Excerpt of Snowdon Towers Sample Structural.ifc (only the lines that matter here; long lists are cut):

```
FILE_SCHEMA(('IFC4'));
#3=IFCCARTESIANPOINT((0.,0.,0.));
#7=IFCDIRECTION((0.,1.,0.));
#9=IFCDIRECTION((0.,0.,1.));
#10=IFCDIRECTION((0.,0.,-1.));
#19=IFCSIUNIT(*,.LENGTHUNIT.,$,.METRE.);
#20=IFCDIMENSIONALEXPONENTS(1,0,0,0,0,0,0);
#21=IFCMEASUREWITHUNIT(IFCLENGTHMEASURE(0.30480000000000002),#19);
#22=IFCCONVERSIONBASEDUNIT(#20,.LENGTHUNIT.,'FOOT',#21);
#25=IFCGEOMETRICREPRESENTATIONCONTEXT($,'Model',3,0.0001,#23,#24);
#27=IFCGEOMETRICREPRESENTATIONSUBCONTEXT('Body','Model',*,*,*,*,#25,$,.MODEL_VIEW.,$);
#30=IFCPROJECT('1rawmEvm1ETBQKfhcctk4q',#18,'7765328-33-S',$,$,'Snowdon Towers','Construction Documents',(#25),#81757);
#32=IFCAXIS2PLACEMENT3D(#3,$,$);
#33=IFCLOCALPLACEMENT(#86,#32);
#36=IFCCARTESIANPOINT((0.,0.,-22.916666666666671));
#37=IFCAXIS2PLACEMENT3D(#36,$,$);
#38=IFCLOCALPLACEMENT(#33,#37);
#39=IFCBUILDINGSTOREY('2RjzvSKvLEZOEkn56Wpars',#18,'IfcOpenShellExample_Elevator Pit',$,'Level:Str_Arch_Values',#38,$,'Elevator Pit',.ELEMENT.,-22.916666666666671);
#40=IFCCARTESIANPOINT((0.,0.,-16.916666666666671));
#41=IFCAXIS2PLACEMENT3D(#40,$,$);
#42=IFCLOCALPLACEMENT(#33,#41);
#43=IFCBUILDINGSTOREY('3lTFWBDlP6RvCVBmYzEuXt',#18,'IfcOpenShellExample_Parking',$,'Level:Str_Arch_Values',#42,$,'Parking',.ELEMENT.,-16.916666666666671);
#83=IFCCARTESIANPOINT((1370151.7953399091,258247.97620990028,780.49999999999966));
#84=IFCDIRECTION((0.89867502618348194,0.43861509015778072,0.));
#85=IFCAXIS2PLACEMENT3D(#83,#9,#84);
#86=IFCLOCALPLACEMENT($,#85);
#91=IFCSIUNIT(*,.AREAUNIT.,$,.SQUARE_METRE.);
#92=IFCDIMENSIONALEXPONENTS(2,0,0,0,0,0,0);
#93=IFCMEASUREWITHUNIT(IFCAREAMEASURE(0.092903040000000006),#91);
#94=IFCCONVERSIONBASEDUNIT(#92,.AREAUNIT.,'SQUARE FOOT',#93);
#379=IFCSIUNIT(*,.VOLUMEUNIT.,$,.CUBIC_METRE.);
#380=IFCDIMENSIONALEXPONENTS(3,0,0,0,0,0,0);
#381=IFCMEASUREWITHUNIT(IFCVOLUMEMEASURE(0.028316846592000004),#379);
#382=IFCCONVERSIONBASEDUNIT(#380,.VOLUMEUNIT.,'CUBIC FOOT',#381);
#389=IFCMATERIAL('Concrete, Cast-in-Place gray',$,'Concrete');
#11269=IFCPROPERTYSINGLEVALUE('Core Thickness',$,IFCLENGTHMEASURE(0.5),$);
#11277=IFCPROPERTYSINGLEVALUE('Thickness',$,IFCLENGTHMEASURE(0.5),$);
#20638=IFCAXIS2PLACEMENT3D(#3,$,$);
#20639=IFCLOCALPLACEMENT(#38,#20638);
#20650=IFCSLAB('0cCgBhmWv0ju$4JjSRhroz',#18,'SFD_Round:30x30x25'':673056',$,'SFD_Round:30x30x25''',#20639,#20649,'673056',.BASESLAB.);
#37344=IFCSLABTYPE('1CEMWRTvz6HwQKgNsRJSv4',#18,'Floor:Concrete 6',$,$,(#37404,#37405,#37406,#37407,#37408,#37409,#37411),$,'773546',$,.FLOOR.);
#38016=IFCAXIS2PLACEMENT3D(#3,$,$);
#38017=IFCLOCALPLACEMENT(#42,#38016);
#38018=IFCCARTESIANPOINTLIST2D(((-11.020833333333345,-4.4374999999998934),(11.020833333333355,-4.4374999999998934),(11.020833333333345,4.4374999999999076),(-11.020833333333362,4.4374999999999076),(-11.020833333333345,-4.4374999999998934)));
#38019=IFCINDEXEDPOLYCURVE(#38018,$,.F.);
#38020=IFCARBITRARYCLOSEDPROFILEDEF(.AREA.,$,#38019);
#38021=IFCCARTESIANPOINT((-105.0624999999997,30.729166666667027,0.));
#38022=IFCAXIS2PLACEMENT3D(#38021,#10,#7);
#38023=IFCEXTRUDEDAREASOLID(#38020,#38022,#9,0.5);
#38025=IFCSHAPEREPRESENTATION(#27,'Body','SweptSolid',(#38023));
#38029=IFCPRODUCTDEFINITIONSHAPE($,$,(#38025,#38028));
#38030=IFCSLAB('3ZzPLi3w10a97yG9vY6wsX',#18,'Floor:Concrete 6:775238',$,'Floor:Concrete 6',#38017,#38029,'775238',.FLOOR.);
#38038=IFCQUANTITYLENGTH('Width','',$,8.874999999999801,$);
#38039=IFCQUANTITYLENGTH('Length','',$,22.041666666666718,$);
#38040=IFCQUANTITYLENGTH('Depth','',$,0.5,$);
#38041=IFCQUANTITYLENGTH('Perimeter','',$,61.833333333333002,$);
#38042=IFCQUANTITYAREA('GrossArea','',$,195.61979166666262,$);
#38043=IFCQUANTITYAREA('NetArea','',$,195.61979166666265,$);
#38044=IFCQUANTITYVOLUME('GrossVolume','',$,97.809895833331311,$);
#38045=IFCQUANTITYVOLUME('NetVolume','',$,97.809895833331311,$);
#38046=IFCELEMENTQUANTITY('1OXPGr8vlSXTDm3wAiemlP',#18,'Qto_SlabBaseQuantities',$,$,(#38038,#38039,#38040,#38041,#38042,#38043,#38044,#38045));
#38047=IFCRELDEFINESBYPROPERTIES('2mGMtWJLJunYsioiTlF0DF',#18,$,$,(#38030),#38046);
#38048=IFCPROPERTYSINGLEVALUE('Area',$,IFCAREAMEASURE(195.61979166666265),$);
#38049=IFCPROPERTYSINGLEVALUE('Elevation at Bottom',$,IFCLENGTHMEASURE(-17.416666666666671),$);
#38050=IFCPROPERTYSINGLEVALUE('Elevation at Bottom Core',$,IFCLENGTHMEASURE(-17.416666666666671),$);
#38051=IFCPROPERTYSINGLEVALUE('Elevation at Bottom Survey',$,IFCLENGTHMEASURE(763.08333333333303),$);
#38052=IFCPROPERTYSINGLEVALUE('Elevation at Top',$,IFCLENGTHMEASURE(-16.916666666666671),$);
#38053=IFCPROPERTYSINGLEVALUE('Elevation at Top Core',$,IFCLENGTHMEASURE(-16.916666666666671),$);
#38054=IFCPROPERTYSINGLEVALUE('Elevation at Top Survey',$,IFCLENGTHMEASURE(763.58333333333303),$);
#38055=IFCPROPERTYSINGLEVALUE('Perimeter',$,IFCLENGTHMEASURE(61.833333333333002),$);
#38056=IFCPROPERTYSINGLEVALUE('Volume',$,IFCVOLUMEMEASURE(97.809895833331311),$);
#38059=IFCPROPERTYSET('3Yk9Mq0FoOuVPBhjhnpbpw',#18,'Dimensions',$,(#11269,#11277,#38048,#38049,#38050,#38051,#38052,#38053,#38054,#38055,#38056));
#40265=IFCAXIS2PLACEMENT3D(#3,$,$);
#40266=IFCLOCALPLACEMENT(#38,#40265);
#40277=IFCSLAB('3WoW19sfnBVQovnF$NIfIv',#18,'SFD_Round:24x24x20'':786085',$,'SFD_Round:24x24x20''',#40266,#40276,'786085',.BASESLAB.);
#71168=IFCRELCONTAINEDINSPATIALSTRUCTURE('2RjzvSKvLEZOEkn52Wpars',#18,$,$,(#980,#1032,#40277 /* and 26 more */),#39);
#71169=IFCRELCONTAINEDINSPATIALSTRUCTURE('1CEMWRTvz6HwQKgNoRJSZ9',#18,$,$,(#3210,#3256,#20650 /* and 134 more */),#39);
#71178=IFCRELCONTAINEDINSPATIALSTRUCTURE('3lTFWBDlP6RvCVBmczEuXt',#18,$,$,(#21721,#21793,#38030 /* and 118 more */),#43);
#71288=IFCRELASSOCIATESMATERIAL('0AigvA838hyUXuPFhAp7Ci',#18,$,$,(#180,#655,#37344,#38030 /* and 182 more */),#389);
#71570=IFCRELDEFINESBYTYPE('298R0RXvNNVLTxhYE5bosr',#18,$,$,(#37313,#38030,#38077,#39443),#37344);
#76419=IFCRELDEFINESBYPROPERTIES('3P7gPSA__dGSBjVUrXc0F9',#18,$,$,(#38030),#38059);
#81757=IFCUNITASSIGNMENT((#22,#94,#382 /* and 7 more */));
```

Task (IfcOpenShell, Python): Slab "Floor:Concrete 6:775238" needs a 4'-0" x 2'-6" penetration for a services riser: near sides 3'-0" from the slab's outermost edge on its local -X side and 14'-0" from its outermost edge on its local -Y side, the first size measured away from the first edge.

```python
import numpy as np
import ifcopenshell
import ifcopenshell.api.feature
import ifcopenshell.api.geometry
import ifcopenshell.api.pset
import ifcopenshell.api.root
import ifcopenshell.geom
import ifcopenshell.util.element
import ifcopenshell.util.placement
import ifcopenshell.util.representation
import ifcopenshell.util.shape
import ifcopenshell.util.unit

model = ifcopenshell.open("Snowdon Towers Sample Structural.ifc")
unit_scale = ifcopenshell.util.unit.calculate_unit_scale(model)
area_scale = ifcopenshell.util.unit.calculate_unit_scale(model, "AREAUNIT")
volume_scale = ifcopenshell.util.unit.calculate_unit_scale(model, "VOLUMEUNIT")
settings = ifcopenshell.geom.settings()


def volume(element):
    """Net volume in cubic metres, openings subtracted."""
    shape = ifcopenshell.geom.create_shape(settings, element)
    return ifcopenshell.util.shape.get_volume(shape.geometry)


slab = model.by_guid("3ZzPLi3w10a97yG9vY6wsX")
before = volume(slab)

# Extent in the slab's own axes, in metres. The edges named are its -X and -Y sides.
slab_shape = ifcopenshell.geom.create_shape(settings, slab)
vertices = ifcopenshell.util.shape.get_vertices(slab_shape.geometry)
x_min, y_min, bottom = vertices.min(axis=0)
top = vertices[:, 2].max()

opening = ifcopenshell.api.root.create_entity(model, ifc_class="IfcOpeningElement", name="Services riser opening", predefined_type="OPENING")
context = ifcopenshell.util.representation.get_context(model, "Model", "Body", "MODEL_VIEW")
width, depth = 1.2192, 0.762
outline = [(0.0, 0.0), (width, 0.0), (width, depth), (0.0, depth), (0.0, 0.0)]
# Overshoot both faces by 50 mm so the cut is clean.
shape = ifcopenshell.api.geometry.add_slab_representation(
    model, context=context, depth=top - bottom + 0.1, polyline=outline
)
ifcopenshell.api.geometry.assign_representation(model, product=opening, representation=shape)

matrix = ifcopenshell.util.placement.get_local_placement(slab.ObjectPlacement)
matrix[:, 3] = matrix @ np.append(np.array([x_min + 0.9144, y_min + 4.2672, bottom - 0.05]) / unit_scale, 1.0)
ifcopenshell.api.geometry.edit_object_placement(model, product=opening, matrix=matrix, is_si=False)
ifcopenshell.api.feature.add_feature(model, feature=opening, element=slab)

after = volume(slab)

# Update the slab's stored quantities.
qto = model.by_id(ifcopenshell.util.element.get_pset(slab, "Qto_SlabBaseQuantities", should_inherit=False)["id"])
ifcopenshell.api.pset.edit_qto(model, qto=qto, properties={
    "NetArea": after / (top - bottom) / area_scale,
    "NetVolume": after / volume_scale,
})
pset = model.by_id(ifcopenshell.util.element.get_pset(slab, "Dimensions", should_inherit=False)["id"])
ifcopenshell.api.pset.edit_pset(model, pset=pset, properties={
    "Area": model.create_entity("IfcAreaMeasure", after / (top - bottom) / area_scale),
    "Volume": model.create_entity("IfcVolumeMeasure", after / volume_scale),
})

print(f"slab volume {before:.3f} -> {after:.3f} m3")

model.write("Snowdon Towers Sample Structural_rev.ifc")
```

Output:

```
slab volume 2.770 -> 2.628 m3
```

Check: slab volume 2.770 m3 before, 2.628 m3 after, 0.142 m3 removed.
